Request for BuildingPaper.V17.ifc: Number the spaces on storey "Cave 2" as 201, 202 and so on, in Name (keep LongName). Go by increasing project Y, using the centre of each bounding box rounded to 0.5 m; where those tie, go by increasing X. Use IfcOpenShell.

First a look at what the model holds.

```python
import ifcopenshell
import ifcopenshell.util.element
import ifcopenshell.util.placement

model = ifcopenshell.open("BuildingPaper.V17.ifc")
print(model.schema)
storey = next(s for s in model.by_type("IfcBuildingStorey") if s.Name == "Cave 2")
spaces = [e for e in ifcopenshell.util.element.get_decomposition(storey) if e.is_a("IfcSpace")]
for e in sorted(spaces, key=lambda e: e.id()):
    origin = ifcopenshell.util.placement.get_local_placement(e.ObjectPlacement)[:3, 3]
    print(e.id(), e.Name, e.LongName, origin.round(2) + 0.0, sep=" | ")
```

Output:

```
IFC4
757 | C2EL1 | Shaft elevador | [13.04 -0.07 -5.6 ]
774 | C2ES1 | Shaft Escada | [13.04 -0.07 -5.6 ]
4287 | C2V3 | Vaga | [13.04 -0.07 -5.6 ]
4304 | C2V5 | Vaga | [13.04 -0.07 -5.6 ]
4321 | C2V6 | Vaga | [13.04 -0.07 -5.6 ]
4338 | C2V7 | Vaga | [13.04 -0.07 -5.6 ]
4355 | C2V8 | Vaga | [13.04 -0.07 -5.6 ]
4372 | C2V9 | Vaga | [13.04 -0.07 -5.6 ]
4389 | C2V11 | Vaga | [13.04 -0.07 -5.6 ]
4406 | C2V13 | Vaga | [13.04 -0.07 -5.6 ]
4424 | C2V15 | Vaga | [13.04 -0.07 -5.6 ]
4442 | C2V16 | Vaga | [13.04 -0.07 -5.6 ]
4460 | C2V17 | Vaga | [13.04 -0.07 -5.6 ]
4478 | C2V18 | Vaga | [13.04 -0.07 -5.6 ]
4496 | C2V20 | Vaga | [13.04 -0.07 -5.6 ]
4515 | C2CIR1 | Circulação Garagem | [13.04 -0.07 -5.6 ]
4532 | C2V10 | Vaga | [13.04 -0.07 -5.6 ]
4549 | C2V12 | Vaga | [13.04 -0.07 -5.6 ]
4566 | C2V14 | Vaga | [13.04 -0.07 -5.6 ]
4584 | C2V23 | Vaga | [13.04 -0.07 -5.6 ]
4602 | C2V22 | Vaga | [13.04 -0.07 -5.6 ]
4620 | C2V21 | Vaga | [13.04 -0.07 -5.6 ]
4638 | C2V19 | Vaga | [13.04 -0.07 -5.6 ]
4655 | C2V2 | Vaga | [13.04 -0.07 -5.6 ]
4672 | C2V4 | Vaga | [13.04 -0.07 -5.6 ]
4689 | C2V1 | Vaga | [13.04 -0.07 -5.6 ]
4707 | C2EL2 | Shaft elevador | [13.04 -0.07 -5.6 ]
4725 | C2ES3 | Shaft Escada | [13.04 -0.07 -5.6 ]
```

```python
import ifcopenshell
import ifcopenshell.geom
import ifcopenshell.util.element
import ifcopenshell.util.shape

model = ifcopenshell.open("BuildingPaper.V17.ifc")
settings = ifcopenshell.geom.settings()
settings.set("use-world-coords", True)


def centre(element):
    shape = ifcopenshell.geom.create_shape(settings, element)
    return ifcopenshell.util.shape.get_bbox_centroid(shape.geometry)


storey = next(s for s in model.by_type("IfcBuildingStorey") if s.Name == "Cave 2")
spaces = [e for e in ifcopenshell.util.element.get_decomposition(storey) if e.is_a("IfcSpace")]

# Insertion points can sit at a corner or the storey origin, so sort by the geometry (in metres).
centres = {e: centre(e) for e in spaces}
spaces.sort(key=lambda e: (round(centres[e][1] / 0.5), centres[e][0]))

for i, e in enumerate(spaces, start=1):
    number = f"2{i:02d}"
    e.Name = number
    print(e.id(), number)

model.write("BuildingPaper.V17_v2.ifc")
```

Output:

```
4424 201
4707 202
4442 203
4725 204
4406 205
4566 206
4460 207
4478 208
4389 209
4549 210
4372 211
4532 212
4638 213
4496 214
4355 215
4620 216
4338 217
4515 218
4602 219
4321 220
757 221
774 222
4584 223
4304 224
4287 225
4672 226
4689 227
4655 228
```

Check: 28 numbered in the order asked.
